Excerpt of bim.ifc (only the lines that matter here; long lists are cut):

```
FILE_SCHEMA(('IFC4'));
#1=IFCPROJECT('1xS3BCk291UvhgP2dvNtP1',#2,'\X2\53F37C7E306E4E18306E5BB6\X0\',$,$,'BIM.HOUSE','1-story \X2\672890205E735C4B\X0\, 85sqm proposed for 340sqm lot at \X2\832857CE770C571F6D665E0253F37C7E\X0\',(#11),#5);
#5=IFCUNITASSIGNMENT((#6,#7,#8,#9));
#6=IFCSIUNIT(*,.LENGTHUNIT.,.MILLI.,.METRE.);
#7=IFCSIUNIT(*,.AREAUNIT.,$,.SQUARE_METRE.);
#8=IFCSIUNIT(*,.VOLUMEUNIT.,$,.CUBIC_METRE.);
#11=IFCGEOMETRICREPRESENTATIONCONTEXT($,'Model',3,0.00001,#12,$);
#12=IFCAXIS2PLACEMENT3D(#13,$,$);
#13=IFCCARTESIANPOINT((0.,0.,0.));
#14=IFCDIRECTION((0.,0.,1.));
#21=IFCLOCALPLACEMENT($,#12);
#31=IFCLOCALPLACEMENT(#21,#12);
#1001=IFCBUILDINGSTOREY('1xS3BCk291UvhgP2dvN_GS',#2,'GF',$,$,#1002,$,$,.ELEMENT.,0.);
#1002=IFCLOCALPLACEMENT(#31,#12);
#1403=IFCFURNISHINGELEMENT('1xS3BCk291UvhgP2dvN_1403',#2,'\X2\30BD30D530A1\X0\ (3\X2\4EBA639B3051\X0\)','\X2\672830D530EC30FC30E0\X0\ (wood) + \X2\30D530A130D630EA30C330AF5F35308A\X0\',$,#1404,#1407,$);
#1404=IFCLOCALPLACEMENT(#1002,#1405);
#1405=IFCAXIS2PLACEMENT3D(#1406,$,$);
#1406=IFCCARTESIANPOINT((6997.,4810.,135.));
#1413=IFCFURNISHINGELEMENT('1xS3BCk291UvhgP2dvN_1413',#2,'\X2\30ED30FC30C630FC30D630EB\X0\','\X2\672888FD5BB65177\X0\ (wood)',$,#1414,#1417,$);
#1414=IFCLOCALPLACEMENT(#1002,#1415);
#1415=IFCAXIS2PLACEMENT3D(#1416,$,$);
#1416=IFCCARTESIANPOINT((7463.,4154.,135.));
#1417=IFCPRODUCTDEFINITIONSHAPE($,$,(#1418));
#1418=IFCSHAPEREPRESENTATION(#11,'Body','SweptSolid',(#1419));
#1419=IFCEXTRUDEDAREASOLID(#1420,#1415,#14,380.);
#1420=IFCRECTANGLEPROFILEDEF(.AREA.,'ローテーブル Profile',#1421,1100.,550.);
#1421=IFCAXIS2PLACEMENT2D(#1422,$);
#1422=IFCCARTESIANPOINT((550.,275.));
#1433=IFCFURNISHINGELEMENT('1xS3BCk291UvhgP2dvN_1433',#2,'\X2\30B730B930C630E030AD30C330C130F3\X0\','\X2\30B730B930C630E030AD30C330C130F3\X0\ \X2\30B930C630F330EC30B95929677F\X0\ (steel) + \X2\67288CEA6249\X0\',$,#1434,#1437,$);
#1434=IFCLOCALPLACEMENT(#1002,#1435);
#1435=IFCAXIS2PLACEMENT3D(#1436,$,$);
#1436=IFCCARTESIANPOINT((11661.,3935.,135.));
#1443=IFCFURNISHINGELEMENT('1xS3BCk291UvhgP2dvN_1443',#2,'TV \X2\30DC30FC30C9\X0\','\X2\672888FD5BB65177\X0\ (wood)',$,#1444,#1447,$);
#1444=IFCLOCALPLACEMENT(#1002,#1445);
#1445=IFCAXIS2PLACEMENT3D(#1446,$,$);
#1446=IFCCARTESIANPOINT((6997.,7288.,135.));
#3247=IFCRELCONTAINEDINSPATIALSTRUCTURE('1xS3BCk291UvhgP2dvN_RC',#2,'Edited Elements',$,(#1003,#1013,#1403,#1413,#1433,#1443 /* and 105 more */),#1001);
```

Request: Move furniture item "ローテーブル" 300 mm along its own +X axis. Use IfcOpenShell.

```python
import ifcopenshell
import ifcopenshell.api.geometry
import ifcopenshell.util.placement
import ifcopenshell.util.unit

model = ifcopenshell.open("bim.ifc")
unit_scale = ifcopenshell.util.unit.calculate_unit_scale(model)

item = model.by_guid("1xS3BCk291UvhgP2dvN_1413")
matrix = ifcopenshell.util.placement.get_local_placement(item.ObjectPlacement)
matrix[:3, 3] += matrix[:3, 0] * 0.3 / unit_scale
ifcopenshell.api.geometry.edit_object_placement(model, product=item, matrix=matrix, is_si=False)

print(ifcopenshell.util.placement.get_local_placement(item.ObjectPlacement).round(3) + 0.0)

model.write("bim-out.ifc")
```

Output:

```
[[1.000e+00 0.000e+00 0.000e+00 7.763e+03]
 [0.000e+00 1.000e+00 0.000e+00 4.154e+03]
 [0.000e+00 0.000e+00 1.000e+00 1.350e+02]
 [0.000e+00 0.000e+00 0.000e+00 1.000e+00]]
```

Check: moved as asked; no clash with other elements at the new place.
